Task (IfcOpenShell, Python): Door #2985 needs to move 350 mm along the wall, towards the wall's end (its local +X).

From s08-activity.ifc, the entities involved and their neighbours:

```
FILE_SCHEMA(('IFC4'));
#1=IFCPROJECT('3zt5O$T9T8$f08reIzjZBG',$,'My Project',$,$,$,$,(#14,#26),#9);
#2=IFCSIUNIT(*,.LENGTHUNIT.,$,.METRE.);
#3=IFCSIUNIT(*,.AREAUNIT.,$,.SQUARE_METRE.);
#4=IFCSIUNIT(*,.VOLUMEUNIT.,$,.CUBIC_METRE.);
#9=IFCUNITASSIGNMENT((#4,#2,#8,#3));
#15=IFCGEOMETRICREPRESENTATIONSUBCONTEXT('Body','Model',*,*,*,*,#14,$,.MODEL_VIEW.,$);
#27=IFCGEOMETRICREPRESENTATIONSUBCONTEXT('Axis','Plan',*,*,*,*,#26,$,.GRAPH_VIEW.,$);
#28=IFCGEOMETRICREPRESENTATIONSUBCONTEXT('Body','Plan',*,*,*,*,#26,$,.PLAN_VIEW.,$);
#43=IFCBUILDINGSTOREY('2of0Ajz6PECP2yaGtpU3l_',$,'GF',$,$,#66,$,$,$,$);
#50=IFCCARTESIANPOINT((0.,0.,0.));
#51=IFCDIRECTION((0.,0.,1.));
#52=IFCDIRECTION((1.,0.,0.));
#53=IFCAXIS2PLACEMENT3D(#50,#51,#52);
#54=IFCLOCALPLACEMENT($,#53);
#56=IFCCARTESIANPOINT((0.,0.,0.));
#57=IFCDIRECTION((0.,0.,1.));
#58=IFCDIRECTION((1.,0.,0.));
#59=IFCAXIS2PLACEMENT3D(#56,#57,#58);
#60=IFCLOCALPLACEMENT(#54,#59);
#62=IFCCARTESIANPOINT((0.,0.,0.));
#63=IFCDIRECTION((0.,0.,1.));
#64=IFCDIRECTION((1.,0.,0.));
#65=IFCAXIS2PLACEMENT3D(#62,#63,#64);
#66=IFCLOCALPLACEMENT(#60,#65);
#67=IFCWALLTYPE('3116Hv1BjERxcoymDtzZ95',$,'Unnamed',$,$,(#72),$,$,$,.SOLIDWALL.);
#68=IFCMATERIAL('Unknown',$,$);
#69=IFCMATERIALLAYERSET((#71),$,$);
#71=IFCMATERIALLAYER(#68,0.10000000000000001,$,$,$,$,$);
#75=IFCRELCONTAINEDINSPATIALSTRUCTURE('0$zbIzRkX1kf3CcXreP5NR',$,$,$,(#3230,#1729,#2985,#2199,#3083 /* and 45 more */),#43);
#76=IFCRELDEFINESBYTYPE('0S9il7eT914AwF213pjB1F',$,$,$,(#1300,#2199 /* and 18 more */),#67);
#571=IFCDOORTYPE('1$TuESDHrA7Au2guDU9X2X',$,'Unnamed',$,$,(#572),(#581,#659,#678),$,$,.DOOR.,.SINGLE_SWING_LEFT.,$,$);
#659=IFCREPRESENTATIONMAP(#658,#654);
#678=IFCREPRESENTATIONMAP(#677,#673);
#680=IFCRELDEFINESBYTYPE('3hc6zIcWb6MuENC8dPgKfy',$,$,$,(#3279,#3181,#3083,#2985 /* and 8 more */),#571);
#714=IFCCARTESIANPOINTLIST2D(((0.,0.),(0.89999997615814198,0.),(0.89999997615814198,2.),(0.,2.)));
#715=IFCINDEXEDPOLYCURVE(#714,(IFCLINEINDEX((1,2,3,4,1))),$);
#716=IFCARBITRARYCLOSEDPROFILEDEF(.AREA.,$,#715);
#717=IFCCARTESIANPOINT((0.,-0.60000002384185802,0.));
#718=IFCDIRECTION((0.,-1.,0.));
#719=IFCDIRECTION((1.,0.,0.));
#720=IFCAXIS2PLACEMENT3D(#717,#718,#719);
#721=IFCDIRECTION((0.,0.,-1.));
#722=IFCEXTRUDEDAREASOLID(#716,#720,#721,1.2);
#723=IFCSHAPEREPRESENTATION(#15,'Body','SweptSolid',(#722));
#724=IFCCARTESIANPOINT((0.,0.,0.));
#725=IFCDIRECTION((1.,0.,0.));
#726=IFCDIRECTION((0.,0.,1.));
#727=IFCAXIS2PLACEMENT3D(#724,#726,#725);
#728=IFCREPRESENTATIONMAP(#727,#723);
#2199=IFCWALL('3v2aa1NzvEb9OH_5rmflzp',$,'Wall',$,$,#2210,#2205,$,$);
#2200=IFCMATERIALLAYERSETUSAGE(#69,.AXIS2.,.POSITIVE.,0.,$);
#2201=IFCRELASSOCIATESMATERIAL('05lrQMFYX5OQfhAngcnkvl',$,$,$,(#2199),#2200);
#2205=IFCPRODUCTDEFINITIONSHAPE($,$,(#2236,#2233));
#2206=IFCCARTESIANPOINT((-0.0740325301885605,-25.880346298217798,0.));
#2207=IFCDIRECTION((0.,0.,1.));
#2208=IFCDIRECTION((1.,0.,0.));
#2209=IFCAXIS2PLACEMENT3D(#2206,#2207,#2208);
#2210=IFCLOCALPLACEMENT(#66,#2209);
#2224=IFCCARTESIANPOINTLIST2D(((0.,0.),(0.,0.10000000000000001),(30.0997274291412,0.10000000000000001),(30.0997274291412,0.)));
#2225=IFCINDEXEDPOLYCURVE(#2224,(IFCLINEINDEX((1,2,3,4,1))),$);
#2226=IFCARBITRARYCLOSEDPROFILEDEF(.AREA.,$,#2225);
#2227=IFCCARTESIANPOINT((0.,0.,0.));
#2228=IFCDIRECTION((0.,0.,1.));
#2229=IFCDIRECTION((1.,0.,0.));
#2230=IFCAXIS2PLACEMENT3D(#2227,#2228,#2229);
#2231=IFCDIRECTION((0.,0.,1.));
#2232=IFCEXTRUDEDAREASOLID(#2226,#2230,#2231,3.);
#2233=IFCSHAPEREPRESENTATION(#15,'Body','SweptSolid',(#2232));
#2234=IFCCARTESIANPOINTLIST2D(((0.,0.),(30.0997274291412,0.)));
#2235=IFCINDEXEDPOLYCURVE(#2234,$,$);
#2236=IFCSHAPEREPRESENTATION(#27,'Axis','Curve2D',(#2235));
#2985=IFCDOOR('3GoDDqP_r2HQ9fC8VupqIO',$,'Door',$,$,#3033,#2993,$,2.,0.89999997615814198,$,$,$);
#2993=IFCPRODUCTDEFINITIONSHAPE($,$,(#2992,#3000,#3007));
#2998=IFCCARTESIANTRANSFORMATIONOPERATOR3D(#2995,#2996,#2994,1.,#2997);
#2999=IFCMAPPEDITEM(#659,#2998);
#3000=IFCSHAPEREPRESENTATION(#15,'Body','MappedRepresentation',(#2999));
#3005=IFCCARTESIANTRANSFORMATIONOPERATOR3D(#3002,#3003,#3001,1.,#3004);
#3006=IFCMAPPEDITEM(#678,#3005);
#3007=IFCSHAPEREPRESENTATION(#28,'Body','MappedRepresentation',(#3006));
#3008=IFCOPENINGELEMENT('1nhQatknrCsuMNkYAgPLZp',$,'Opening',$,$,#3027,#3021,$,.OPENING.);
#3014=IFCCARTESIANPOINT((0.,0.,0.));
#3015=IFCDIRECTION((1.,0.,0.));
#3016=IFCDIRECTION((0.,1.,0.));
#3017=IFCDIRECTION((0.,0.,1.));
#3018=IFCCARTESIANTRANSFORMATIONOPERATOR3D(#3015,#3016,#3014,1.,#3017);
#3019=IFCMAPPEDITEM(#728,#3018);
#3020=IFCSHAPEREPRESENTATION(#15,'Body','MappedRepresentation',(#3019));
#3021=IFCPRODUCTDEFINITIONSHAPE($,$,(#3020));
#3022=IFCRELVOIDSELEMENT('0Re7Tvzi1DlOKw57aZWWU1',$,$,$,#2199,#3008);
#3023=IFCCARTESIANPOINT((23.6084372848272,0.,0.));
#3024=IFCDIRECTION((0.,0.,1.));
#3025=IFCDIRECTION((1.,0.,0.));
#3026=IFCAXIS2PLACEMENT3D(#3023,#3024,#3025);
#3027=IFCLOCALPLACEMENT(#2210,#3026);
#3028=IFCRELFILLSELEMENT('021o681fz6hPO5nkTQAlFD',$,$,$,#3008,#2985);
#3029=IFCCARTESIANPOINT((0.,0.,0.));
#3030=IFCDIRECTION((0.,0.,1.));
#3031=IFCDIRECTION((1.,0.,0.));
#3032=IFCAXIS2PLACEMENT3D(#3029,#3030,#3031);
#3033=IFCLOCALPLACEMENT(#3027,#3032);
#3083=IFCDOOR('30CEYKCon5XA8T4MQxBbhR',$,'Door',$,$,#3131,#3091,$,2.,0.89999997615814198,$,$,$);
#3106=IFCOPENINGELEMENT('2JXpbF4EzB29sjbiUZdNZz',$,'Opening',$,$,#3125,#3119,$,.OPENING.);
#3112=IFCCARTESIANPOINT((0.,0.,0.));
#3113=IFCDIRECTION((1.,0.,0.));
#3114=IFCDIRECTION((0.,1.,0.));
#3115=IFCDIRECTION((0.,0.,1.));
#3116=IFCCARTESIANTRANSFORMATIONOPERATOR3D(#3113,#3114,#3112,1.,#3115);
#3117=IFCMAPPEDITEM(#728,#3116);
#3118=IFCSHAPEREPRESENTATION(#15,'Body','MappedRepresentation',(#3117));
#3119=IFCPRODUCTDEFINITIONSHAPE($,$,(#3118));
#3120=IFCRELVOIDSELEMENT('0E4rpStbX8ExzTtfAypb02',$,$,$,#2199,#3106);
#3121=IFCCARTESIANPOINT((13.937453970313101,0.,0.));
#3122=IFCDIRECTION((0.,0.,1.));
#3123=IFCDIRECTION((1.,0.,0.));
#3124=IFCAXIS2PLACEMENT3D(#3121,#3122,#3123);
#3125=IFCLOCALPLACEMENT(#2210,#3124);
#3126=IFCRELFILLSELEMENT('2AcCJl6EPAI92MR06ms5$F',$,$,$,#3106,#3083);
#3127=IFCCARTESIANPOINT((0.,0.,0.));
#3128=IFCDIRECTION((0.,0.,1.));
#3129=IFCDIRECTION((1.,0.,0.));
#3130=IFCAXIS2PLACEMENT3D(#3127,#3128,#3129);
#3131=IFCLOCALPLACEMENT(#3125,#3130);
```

```python
import ifcopenshell
import ifcopenshell.api.geometry
import ifcopenshell.util.placement
import ifcopenshell.util.unit

model = ifcopenshell.open("s08-activity.ifc")
unit_scale = ifcopenshell.util.unit.calculate_unit_scale(model)

door = model.by_guid("3GoDDqP_r2HQ9fC8VupqIO")
opening = door.FillsVoids[0].RelatingOpeningElement
wall = opening.VoidsElements[0].RelatingBuildingElement

wall_matrix = ifcopenshell.util.placement.get_local_placement(wall.ObjectPlacement)
shift = wall_matrix[:3, 0] * 0.35 / unit_scale
before = ifcopenshell.util.placement.get_local_placement(door.ObjectPlacement)[:3, 3].copy()

# The door is placed relative to its opening, so it follows when the opening moves.
matrix = ifcopenshell.util.placement.get_local_placement(opening.ObjectPlacement)
matrix[:3, 3] += shift
ifcopenshell.api.geometry.edit_object_placement(
    model, product=opening, matrix=matrix, is_si=False, should_transform_children=True
)

after = ifcopenshell.util.placement.get_local_placement(door.ObjectPlacement)[:3, 3]
print("door moved by", (after - before).round(3) + 0.0)

model.write("s08-activity_edited.ifc")
```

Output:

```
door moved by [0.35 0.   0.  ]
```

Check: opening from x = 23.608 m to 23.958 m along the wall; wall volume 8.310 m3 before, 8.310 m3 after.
